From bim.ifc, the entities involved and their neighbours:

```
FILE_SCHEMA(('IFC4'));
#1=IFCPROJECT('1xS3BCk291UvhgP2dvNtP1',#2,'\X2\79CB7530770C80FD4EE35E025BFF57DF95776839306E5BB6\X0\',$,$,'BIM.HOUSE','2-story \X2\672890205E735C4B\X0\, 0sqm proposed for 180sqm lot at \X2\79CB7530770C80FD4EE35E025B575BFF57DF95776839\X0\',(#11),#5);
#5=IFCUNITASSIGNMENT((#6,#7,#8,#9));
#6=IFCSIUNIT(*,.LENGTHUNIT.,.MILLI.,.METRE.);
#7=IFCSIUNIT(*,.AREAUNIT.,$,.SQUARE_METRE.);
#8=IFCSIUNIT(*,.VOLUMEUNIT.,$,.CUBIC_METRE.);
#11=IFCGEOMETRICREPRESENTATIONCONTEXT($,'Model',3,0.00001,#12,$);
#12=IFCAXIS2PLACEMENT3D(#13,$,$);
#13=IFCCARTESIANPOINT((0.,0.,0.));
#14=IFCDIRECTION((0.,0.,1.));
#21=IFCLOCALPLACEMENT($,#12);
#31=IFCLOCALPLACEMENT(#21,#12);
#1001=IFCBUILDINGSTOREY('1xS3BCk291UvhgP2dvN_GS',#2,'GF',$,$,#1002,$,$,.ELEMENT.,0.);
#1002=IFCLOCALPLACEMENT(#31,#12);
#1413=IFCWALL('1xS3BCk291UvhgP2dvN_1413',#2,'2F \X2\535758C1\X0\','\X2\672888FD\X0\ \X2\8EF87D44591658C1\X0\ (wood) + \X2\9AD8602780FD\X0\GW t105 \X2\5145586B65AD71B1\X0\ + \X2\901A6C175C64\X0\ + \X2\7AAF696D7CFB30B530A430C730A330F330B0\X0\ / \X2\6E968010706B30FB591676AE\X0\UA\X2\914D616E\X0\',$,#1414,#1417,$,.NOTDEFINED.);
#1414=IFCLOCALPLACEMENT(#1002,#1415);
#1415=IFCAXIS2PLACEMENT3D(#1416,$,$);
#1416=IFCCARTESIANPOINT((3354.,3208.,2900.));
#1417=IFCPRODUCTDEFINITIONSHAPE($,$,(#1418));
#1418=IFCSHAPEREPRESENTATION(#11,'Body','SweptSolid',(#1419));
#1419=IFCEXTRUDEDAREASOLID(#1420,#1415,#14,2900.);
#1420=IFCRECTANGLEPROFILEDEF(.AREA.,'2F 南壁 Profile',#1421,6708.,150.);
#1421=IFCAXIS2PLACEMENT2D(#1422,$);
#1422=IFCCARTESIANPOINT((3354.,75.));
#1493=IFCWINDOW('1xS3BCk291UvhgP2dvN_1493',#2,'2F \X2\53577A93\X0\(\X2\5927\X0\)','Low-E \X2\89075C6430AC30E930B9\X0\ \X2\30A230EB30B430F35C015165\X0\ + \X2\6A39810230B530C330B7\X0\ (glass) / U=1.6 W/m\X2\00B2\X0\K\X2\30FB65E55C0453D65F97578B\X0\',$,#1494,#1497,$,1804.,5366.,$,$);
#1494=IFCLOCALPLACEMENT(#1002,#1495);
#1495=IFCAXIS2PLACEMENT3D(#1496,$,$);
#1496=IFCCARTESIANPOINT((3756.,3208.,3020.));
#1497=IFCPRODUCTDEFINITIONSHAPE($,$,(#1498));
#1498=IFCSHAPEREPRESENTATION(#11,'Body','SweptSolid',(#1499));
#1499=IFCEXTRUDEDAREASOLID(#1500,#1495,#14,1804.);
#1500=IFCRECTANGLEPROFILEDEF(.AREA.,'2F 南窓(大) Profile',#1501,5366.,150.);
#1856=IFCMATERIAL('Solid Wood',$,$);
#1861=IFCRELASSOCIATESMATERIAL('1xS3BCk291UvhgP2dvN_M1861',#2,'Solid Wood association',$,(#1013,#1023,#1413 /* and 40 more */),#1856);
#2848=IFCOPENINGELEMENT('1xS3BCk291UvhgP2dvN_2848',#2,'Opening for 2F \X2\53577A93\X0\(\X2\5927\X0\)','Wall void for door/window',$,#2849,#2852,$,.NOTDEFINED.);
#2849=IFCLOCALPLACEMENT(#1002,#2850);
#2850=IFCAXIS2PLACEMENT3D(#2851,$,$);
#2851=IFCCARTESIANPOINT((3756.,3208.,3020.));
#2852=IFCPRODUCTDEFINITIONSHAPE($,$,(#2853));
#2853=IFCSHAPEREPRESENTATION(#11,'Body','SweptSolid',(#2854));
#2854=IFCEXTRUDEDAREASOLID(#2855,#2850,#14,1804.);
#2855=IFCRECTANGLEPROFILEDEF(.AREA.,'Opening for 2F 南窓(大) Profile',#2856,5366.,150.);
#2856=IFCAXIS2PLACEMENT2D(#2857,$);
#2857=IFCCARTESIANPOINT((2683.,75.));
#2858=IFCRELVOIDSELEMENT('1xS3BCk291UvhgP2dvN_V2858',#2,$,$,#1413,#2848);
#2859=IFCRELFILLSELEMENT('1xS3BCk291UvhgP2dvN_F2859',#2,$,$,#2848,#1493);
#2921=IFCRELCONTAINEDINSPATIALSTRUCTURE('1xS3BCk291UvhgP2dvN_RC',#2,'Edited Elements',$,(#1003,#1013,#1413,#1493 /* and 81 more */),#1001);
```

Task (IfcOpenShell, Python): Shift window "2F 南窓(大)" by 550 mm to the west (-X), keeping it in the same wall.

```python
import ifcopenshell
import ifcopenshell.api.geometry
import ifcopenshell.util.placement

model = ifcopenshell.open("bim.ifc")

window = model.by_guid("1xS3BCk291UvhgP2dvN_1493")
opening = window.FillsVoids[0].RelatingOpeningElement
wall = opening.VoidsElements[0].RelatingBuildingElement

wall_matrix = ifcopenshell.util.placement.get_local_placement(wall.ObjectPlacement)
shift = wall_matrix[:3, 0] * -550.0
before = ifcopenshell.util.placement.get_local_placement(window.ObjectPlacement)[:3, 3].copy()

# The window is not placed relative to its opening, so move both.
for product in (opening, window):
    matrix = ifcopenshell.util.placement.get_local_placement(product.ObjectPlacement)
    matrix[:3, 3] += shift
    ifcopenshell.api.geometry.edit_object_placement(model, product=product, matrix=matrix, is_si=False)

after = ifcopenshell.util.placement.get_local_placement(window.ObjectPlacement)[:3, 3]
print("window moved by", (after - before).round(3) + 0.0)

model.write("bim_edited.ifc")
```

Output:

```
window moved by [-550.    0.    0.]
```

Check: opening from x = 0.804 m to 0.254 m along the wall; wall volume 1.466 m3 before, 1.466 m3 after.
